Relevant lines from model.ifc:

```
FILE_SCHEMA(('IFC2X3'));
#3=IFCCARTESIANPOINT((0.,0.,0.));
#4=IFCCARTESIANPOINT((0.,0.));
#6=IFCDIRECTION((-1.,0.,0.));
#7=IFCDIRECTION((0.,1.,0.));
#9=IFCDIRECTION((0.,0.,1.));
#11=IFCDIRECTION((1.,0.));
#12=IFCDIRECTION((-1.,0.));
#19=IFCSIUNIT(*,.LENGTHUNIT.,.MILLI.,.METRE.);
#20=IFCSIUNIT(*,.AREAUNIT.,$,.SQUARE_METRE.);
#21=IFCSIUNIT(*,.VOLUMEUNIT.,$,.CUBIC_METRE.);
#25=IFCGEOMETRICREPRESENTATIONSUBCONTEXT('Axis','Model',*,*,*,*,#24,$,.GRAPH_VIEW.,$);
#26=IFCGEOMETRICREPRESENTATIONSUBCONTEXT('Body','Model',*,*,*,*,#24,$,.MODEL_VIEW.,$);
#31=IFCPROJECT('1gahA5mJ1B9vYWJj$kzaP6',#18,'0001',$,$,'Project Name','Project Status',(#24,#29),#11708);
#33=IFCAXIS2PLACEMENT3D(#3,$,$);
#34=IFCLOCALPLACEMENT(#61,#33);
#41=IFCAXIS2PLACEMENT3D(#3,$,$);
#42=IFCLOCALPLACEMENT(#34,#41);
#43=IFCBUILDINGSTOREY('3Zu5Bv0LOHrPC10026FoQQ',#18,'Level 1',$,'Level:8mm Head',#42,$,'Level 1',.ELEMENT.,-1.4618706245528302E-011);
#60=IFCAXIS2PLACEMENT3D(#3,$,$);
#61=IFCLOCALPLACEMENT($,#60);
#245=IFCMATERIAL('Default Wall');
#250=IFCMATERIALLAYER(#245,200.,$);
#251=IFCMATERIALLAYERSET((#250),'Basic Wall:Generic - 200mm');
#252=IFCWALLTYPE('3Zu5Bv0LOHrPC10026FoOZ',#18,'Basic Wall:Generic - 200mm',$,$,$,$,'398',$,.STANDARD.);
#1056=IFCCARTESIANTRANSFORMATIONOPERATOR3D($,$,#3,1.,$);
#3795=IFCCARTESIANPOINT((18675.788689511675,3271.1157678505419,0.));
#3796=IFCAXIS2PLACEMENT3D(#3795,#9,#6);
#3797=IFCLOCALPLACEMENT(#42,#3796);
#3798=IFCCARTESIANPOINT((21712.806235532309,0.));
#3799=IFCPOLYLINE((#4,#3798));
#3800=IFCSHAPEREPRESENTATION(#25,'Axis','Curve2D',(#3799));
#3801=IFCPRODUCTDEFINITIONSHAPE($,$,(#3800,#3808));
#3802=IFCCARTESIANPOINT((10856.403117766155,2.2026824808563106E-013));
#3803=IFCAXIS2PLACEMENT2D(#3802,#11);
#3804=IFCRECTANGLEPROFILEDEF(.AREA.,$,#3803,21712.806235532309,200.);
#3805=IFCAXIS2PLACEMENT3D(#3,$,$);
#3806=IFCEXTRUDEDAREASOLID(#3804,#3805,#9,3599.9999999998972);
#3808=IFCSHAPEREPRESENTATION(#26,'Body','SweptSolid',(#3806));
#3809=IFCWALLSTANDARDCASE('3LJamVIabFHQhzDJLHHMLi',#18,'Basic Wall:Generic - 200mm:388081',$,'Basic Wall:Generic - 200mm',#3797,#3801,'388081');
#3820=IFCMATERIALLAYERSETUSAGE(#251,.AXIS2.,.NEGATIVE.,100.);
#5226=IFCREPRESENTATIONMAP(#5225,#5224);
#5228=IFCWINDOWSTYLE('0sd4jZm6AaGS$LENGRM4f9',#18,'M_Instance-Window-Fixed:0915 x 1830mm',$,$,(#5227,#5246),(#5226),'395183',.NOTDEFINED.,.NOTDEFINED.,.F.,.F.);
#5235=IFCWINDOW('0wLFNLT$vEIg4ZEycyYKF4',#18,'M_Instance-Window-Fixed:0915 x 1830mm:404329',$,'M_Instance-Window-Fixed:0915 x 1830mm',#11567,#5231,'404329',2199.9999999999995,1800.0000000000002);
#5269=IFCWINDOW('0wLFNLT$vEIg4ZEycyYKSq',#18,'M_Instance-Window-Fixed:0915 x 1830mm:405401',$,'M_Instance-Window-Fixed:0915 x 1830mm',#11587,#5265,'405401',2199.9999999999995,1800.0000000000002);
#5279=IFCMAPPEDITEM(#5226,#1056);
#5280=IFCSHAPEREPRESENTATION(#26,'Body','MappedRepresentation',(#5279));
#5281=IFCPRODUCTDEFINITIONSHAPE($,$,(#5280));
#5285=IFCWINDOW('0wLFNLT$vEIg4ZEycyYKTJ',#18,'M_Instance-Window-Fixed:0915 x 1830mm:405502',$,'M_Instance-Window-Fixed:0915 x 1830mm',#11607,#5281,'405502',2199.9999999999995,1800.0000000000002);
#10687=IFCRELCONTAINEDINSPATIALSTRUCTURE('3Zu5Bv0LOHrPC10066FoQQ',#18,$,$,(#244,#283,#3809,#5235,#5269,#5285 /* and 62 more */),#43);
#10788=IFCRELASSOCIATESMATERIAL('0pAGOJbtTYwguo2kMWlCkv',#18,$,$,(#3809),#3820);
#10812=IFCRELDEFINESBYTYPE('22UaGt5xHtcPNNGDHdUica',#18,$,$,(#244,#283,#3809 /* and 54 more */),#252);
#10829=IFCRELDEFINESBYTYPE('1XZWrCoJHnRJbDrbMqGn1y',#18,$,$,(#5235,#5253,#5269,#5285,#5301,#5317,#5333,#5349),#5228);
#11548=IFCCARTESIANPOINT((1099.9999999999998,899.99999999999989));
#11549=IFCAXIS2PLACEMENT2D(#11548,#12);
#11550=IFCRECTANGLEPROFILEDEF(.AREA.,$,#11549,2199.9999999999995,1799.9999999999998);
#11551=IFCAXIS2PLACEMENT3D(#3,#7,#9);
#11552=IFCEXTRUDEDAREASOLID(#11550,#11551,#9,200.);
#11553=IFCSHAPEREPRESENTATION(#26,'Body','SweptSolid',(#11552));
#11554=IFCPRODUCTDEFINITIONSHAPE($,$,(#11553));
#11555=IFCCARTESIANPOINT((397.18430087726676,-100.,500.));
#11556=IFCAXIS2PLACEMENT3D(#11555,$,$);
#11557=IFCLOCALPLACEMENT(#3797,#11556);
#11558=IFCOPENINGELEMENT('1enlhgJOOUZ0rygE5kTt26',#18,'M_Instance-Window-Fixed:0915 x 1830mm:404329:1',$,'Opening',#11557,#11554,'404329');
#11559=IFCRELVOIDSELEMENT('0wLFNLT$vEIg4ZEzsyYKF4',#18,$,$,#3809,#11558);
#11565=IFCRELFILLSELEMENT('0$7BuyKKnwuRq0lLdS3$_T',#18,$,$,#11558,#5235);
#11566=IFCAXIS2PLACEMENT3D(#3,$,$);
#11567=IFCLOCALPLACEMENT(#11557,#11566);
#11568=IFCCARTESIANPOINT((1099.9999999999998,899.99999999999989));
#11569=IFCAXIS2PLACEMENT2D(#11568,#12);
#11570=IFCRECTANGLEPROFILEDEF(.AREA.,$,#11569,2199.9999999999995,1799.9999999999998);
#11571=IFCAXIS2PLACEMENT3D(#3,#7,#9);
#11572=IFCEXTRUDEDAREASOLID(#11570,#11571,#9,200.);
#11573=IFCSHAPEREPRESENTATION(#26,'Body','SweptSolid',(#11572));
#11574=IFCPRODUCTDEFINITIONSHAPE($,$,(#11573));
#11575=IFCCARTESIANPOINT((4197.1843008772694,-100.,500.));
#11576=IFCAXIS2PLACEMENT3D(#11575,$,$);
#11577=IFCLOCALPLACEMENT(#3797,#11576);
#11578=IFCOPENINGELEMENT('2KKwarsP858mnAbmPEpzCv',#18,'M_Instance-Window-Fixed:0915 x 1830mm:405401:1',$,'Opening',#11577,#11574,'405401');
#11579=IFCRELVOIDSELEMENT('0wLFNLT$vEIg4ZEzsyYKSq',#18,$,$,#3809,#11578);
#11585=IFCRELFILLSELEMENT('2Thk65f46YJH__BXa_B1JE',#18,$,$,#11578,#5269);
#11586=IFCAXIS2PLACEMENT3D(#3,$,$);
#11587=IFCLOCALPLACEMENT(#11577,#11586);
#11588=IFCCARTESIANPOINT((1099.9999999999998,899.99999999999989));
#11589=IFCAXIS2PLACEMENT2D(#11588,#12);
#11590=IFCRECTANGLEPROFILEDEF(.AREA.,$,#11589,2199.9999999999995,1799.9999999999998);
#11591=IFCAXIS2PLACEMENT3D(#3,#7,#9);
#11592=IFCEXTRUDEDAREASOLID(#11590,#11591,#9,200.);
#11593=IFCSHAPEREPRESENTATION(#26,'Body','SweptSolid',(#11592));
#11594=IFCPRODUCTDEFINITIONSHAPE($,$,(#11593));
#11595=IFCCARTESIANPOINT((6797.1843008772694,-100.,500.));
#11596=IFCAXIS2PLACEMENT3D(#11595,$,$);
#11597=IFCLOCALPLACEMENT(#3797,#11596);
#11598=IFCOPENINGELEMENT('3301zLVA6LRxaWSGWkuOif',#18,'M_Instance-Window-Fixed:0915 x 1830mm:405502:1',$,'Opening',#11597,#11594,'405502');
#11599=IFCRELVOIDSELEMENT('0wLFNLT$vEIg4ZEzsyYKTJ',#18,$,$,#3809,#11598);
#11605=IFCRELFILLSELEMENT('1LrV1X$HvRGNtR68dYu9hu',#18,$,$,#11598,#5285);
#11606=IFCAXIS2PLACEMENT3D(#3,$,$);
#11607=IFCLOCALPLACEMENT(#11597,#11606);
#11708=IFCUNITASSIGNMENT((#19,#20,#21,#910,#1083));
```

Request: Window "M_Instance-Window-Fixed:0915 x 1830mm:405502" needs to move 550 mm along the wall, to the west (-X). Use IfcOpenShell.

```python
import ifcopenshell
import ifcopenshell.api.geometry
import ifcopenshell.util.placement
import ifcopenshell.util.unit

model = ifcopenshell.open("model.ifc")
unit_scale = ifcopenshell.util.unit.calculate_unit_scale(model)

window = model.by_id(5285)
opening = window.FillsVoids[0].RelatingOpeningElement
wall = opening.VoidsElements[0].RelatingBuildingElement

wall_matrix = ifcopenshell.util.placement.get_local_placement(wall.ObjectPlacement)
shift = wall_matrix[:3, 0] * 0.55 / unit_scale
before = ifcopenshell.util.placement.get_local_placement(window.ObjectPlacement)[:3, 3].copy()

# The window is placed relative to its opening, so it follows when the opening moves.
matrix = ifcopenshell.util.placement.get_local_placement(opening.ObjectPlacement)
matrix[:3, 3] += shift
ifcopenshell.api.geometry.edit_object_placement(
    model, product=opening, matrix=matrix, is_si=False, should_transform_children=True
)

after = ifcopenshell.util.placement.get_local_placement(window.ObjectPlacement)[:3, 3]
print("window moved by", (after - before).round(3) + 0.0)

model.write("model-out.ifc")
```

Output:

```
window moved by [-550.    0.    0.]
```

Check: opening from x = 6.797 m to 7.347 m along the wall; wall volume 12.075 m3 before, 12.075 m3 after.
